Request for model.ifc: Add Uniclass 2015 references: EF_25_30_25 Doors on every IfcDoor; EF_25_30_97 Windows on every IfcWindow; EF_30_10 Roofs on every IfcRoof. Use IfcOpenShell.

First a look at what the model holds.

```python
import ifcopenshell

model = ifcopenshell.open("model.ifc")
print(model.schema)
print("classifications:", [c.Name for c in model.by_type("IfcClassification")])
for ifc_class in ("IfcDoor", "IfcRoof", "IfcStair", "IfcWall", "IfcWindow"):
    print(ifc_class, len(model.by_type(ifc_class)))
```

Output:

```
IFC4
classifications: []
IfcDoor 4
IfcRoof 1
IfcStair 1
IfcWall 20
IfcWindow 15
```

```python
import ifcopenshell
import ifcopenshell.api.classification

model = ifcopenshell.open("model.ifc")

system = ifcopenshell.api.classification.add_classification(model, classification="Uniclass 2015")

codes = {
    "IfcDoor": ("EF_25_30_25", "Doors"),
    "IfcWindow": ("EF_25_30_97", "Windows"),
    "IfcRoof": ("EF_30_10", "Roofs"),
}
for ifc_class, (code, name) in codes.items():
    products = model.by_type(ifc_class)
    ifcopenshell.api.classification.add_reference(
        model, products=products, classification=system, identification=code, name=name
    )
    print(code, len(products))

model.write("model_v2.ifc")
```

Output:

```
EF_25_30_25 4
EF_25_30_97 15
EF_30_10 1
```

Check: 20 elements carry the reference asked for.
